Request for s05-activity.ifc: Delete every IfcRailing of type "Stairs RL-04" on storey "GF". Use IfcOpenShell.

First a look at what the model holds.

```python
import ifcopenshell
import ifcopenshell.util.element

model = ifcopenshell.open("s05-activity.ifc")
print(model.schema)
storey = next(s for s in model.by_type("IfcBuildingStorey") if s.Name == "GF")
railings = [e for e in ifcopenshell.util.element.get_decomposition(storey) if e.is_a("IfcRailing")]
seen = {}
for e in railings:
    element_type = ifcopenshell.util.element.get_type(e)
    name = element_type.Name if element_type not in (None, e) else None
    seen[name] = seen.get(name, 0) + 1
for name, count in sorted(seen.items(), key=str):
    print(count, "x", name)
```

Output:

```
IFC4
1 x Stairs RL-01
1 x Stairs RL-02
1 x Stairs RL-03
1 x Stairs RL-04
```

```python
import ifcopenshell
import ifcopenshell.api.root
import ifcopenshell.util.element

model = ifcopenshell.open("s05-activity.ifc")

storey = next(s for s in model.by_type("IfcBuildingStorey") if s.Name == "GF")
railings = [e for e in ifcopenshell.util.element.get_decomposition(storey) if e.is_a("IfcRailing")]
targets = [e for e in railings if (t := ifcopenshell.util.element.get_type(e)) not in (None, e) and t.Name == "Stairs RL-04"]

for e in targets:
    ifcopenshell.api.root.remove_product(model, product=e)
print(len(targets), "removed")

model.write("s05-activity-out.ifc")
```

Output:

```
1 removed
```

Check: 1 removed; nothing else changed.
